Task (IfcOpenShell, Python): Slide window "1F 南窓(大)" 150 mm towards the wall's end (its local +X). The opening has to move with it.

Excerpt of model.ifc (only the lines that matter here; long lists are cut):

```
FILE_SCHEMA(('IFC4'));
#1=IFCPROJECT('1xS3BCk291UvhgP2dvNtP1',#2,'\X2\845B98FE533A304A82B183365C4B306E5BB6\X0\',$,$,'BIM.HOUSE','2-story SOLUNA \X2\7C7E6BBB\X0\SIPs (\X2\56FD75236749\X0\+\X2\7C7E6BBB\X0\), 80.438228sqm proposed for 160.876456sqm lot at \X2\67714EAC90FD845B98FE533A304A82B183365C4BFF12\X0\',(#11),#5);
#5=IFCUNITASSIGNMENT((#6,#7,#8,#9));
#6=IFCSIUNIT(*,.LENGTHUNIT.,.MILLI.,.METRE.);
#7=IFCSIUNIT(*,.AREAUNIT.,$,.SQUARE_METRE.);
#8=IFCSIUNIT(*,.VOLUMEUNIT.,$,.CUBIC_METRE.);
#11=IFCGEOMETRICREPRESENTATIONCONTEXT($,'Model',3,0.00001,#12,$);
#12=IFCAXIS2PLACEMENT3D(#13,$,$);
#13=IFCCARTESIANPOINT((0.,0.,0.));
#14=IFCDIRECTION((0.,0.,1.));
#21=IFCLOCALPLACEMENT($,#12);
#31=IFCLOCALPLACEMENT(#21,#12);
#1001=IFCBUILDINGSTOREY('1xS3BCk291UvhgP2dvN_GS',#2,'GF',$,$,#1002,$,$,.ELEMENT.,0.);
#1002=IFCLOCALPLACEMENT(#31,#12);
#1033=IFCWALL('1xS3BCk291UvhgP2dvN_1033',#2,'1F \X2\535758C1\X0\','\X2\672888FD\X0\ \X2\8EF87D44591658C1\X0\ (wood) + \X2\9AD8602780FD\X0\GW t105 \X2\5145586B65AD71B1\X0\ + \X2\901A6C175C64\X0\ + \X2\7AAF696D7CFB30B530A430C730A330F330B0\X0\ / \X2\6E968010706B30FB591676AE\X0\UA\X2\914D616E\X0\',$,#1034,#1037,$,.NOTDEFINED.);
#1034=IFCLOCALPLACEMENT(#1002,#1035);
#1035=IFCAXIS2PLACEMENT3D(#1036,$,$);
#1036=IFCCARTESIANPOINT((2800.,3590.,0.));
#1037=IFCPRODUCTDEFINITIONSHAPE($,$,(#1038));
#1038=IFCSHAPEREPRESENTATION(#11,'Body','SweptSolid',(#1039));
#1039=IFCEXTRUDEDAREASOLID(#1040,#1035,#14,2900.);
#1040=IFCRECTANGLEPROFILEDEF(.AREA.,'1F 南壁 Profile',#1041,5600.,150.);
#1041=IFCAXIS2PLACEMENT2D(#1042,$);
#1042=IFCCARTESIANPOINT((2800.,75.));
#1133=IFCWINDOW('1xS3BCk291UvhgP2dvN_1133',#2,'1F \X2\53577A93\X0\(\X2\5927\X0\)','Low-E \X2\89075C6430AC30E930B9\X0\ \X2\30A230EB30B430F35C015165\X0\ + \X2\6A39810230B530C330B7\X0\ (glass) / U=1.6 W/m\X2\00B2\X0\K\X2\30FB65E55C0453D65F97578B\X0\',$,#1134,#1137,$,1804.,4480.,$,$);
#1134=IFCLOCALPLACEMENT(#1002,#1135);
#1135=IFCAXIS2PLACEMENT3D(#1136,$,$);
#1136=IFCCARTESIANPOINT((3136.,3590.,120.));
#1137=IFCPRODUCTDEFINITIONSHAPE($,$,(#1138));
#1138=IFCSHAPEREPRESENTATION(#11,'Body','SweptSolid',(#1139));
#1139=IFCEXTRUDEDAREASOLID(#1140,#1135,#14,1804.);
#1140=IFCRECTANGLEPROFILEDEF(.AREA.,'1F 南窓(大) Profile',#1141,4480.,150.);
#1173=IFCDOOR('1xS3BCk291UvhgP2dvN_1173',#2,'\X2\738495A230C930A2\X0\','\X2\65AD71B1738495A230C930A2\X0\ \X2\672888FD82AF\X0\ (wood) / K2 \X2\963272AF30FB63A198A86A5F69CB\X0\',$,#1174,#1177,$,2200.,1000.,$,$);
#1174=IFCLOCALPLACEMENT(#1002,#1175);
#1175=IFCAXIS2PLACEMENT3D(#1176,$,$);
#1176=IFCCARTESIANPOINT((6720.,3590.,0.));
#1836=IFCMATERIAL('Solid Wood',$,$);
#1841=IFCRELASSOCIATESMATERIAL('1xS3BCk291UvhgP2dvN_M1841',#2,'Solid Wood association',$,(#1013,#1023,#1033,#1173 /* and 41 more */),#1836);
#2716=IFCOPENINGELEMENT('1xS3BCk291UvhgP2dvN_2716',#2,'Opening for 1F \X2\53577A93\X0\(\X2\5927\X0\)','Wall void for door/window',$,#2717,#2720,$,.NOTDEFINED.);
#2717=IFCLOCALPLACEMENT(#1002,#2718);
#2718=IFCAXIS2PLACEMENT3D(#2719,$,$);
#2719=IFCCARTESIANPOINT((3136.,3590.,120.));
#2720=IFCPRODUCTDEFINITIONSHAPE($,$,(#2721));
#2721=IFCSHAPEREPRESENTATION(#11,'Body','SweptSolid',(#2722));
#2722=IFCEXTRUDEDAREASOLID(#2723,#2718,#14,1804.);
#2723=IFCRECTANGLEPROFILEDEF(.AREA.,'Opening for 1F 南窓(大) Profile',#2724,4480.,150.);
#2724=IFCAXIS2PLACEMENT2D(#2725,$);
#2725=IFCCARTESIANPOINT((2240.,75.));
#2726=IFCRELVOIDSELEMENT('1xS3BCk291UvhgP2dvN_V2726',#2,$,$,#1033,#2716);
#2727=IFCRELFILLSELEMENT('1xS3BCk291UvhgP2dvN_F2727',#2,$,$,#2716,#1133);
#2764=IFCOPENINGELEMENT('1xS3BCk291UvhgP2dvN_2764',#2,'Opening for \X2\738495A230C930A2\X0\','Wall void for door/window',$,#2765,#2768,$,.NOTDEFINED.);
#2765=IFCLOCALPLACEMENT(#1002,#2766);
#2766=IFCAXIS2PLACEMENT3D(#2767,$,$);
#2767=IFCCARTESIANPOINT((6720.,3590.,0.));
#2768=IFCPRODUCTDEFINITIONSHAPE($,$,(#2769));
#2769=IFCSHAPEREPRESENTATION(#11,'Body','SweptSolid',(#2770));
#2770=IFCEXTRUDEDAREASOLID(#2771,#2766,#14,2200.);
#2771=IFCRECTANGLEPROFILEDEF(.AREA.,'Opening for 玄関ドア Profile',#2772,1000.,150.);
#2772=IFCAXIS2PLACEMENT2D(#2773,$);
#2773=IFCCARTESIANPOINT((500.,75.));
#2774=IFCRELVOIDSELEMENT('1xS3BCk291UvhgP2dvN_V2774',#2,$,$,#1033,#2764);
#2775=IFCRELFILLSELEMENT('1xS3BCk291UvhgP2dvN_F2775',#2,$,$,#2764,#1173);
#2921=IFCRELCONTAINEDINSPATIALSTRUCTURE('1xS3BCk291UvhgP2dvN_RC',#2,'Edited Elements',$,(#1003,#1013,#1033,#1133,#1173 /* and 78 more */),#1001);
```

```python
import ifcopenshell
import ifcopenshell.api.geometry
import ifcopenshell.util.placement
import ifcopenshell.util.unit

model = ifcopenshell.open("model.ifc")
unit_scale = ifcopenshell.util.unit.calculate_unit_scale(model)

window = model.by_guid("1xS3BCk291UvhgP2dvN_1133")
opening = window.FillsVoids[0].RelatingOpeningElement
wall = opening.VoidsElements[0].RelatingBuildingElement

wall_matrix = ifcopenshell.util.placement.get_local_placement(wall.ObjectPlacement)
shift = wall_matrix[:3, 0] * 0.15 / unit_scale
before = ifcopenshell.util.placement.get_local_placement(window.ObjectPlacement)[:3, 3].copy()

# The window is not placed relative to its opening, so move both.
for product in (opening, window):
    matrix = ifcopenshell.util.placement.get_local_placement(product.ObjectPlacement)
    matrix[:3, 3] += shift
    ifcopenshell.api.geometry.edit_object_placement(model, product=product, matrix=matrix, is_si=False)

after = ifcopenshell.util.placement.get_local_placement(window.ObjectPlacement)[:3, 3]
print("window moved by", (after - before).round(3) + 0.0)

model.write("model_v2.ifc")
```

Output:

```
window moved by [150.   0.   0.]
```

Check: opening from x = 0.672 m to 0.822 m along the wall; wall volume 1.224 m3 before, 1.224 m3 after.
